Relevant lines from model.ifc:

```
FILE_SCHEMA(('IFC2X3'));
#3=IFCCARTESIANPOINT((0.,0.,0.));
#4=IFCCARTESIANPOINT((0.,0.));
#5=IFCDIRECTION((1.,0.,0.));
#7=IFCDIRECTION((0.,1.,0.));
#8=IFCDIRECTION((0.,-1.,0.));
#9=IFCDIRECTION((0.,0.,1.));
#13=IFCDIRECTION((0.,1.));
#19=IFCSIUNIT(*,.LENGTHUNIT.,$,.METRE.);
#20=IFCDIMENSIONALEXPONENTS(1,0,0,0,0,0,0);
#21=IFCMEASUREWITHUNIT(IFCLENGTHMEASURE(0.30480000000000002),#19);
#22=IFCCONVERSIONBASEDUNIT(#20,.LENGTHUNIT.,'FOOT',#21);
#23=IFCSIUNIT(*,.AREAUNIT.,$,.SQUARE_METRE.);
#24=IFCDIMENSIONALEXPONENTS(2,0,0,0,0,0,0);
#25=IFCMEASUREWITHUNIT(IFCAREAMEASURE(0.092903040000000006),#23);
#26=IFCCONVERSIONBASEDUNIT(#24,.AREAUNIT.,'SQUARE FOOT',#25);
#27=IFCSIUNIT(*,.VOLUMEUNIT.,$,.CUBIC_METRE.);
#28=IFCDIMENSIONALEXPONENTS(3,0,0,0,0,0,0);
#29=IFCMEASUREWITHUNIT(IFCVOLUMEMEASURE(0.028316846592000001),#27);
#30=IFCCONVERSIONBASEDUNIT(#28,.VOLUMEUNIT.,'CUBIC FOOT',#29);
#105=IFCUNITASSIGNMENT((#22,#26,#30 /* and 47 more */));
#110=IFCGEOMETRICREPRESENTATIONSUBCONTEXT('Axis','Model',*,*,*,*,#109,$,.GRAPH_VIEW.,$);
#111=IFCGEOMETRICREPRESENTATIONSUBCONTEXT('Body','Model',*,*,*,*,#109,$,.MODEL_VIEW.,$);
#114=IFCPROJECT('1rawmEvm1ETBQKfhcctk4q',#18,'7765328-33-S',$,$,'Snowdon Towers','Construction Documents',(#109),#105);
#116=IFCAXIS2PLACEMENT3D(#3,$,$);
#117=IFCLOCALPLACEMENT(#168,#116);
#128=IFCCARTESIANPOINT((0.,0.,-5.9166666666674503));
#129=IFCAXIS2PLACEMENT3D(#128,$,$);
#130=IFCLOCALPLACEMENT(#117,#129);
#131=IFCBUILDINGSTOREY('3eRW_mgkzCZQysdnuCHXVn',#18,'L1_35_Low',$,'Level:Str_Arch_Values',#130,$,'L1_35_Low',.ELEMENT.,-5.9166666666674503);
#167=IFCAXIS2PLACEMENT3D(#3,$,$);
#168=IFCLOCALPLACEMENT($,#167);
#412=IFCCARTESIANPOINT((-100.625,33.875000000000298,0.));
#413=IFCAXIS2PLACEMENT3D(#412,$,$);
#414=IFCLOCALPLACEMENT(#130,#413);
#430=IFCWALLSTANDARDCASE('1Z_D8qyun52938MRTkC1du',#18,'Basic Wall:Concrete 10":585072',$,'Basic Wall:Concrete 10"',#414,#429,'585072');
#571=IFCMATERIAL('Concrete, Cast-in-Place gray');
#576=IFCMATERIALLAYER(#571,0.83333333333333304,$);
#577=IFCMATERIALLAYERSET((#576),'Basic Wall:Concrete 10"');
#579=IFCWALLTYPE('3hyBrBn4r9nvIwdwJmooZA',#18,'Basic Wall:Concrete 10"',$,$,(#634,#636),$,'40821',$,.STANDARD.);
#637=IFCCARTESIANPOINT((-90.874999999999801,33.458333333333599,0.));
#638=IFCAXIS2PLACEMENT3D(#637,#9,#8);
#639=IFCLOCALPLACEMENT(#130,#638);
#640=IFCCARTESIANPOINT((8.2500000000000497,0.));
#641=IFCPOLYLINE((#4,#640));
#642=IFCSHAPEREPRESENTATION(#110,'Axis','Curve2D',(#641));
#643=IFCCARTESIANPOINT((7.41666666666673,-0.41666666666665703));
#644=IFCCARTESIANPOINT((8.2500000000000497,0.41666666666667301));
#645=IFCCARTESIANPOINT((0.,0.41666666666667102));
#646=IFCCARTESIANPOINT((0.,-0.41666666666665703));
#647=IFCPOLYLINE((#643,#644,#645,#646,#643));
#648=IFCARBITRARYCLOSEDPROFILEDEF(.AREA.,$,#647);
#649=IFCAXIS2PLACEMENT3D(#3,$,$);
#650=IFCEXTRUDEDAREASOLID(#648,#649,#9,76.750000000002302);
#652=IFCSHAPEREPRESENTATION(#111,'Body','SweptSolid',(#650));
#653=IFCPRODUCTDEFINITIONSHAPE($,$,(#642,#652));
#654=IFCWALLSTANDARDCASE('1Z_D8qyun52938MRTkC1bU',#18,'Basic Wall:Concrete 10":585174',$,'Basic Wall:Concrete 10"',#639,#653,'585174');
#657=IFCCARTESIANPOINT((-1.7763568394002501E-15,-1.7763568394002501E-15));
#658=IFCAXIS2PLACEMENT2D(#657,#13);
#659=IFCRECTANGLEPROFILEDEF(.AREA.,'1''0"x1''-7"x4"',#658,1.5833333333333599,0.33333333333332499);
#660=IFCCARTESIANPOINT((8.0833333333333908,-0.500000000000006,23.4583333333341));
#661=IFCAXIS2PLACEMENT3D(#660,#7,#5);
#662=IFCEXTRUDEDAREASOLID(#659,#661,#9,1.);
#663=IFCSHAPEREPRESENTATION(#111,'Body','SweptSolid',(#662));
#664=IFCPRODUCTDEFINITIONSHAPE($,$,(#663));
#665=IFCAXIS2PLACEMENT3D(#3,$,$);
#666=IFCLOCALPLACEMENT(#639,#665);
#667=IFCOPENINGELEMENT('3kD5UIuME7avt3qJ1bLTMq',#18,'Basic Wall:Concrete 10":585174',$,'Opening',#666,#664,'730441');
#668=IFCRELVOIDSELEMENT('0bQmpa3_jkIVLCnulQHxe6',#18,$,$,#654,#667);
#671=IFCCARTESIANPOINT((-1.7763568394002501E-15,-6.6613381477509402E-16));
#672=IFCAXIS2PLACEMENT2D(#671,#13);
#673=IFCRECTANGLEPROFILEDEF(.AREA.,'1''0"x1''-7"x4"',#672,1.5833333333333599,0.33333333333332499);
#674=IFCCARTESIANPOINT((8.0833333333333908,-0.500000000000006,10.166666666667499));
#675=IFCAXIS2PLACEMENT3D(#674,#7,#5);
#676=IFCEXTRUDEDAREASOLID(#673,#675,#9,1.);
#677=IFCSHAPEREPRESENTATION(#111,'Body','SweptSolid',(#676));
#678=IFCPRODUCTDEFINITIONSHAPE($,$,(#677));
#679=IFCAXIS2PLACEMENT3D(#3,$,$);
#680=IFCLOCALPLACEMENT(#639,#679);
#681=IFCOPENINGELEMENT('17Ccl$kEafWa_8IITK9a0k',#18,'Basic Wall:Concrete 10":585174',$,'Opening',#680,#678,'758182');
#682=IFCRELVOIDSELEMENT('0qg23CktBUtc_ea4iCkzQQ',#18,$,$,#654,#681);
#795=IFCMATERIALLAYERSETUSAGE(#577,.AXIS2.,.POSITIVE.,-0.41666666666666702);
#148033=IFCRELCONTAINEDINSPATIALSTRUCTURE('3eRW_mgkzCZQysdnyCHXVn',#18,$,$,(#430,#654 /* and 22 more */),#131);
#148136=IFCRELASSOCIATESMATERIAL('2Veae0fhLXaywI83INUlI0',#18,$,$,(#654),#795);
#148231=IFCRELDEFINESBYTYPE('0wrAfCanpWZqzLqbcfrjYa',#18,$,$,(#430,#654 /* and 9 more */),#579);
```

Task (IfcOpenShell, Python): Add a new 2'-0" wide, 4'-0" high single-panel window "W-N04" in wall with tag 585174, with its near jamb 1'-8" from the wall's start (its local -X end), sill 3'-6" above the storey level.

```python
import numpy as np
import ifcopenshell
import ifcopenshell.api.feature
import ifcopenshell.api.geometry
import ifcopenshell.api.root
import ifcopenshell.api.spatial
import ifcopenshell.api.type
import ifcopenshell.geom
import ifcopenshell.util.element
import ifcopenshell.util.placement
import ifcopenshell.util.representation
import ifcopenshell.util.shape
import ifcopenshell.util.unit

model = ifcopenshell.open("model.ifc")
unit_scale = ifcopenshell.util.unit.calculate_unit_scale(model)
settings = ifcopenshell.geom.settings()


def volume(element):
    """Net volume in cubic metres, openings subtracted."""
    shape = ifcopenshell.geom.create_shape(settings, element)
    return ifcopenshell.util.shape.get_volume(shape.geometry)


wall = model.by_guid("1Z_D8qyun52938MRTkC1bU")
storey = ifcopenshell.util.element.get_container(wall, ifc_class="IfcBuildingStorey")
context = ifcopenshell.util.representation.get_context(model, "Model", "Body", "MODEL_VIEW")
before = volume(wall)

width, height, from_end, sill = 0.6096, 1.2192, 0.508, 1.0668  # metres

# The wall runs along its own X axis, and the end named is its -X end.
wall_shape = ifcopenshell.geom.create_shape(settings, wall)
x, y, z = ifcopenshell.util.shape.get_vertices(wall_shape.geometry).T
start = x.min() + from_end
face, thickness = float(y.min()), float(y.max() - y.min())
wall_matrix = ifcopenshell.util.placement.get_local_placement(wall.ObjectPlacement)
level = ifcopenshell.util.placement.get_local_placement(storey.ObjectPlacement)[2, 3]


def in_wall(x, y):
    """Placement at x, y metres in the wall's axes, at sill height."""
    matrix = wall_matrix.copy()
    matrix[:, 3] = wall_matrix @ np.array([x / unit_scale, y / unit_scale, 0.0, 1.0])
    matrix[2, 3] = level + sill / unit_scale
    return matrix


# Opening: a box that overshoots both wall faces by 50 mm.
opening = ifcopenshell.api.root.create_entity(model, ifc_class="IfcOpeningElement")
box = ifcopenshell.api.geometry.add_wall_representation(
    model, context=context, length=width, height=height, thickness=thickness + 0.1
)
ifcopenshell.api.geometry.assign_representation(model, product=opening, representation=box)
ifcopenshell.api.geometry.edit_object_placement(model, product=opening, matrix=in_wall(start, face - 0.05), is_si=False)
ifcopenshell.api.feature.add_feature(model, feature=opening, element=wall)

window = ifcopenshell.api.root.create_entity(model, ifc_class="IfcWindow", name="W-N04")
window.OverallWidth, window.OverallHeight = width / unit_scale, height / unit_scale
body = ifcopenshell.api.geometry.add_window_representation(
    model,
    context=context,
    overall_width=window.OverallWidth,
    overall_height=window.OverallHeight,
    partition_type="SINGLE_PANEL",
)
ifcopenshell.api.geometry.assign_representation(model, product=window, representation=body)
ifcopenshell.api.spatial.assign_container(model, products=[window], relating_structure=storey)
fills = ifcopenshell.api.feature.add_filling(model, opening=opening, element=window)
fills.OwnerHistory = window.OwnerHistory  # required in IFC2X3

# IFC2X3 keeps the operation on the window style.
style = ifcopenshell.api.root.create_entity(model, ifc_class="IfcWindowStyle", name="W-N04")
style.OperationType, style.ConstructionType = "SINGLE_PANEL", "NOTDEFINED"
style.ParameterTakesPrecedence = style.Sizeable = False
ifcopenshell.api.type.assign_type(model, related_objects=[window], relating_type=style)

# Centre the window in the wall's thickness.
ifcopenshell.api.geometry.edit_object_placement(model, product=window, matrix=in_wall(start, face), is_si=False)
window_shape = ifcopenshell.geom.create_shape(settings, window)
depth = ifcopenshell.util.shape.get_vertices(window_shape.geometry)[:, 1]
offset = face + thickness / 2 - (depth.min() + depth.max()) / 2
ifcopenshell.api.geometry.edit_object_placement(model, product=window, matrix=in_wall(start, offset), is_si=False)

after = volume(wall)

print(f"wall volume {before:.3f} -> {after:.3f} m3")

model.write("model_rev.ifc")
```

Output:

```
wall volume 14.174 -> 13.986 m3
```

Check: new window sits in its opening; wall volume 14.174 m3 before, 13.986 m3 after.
